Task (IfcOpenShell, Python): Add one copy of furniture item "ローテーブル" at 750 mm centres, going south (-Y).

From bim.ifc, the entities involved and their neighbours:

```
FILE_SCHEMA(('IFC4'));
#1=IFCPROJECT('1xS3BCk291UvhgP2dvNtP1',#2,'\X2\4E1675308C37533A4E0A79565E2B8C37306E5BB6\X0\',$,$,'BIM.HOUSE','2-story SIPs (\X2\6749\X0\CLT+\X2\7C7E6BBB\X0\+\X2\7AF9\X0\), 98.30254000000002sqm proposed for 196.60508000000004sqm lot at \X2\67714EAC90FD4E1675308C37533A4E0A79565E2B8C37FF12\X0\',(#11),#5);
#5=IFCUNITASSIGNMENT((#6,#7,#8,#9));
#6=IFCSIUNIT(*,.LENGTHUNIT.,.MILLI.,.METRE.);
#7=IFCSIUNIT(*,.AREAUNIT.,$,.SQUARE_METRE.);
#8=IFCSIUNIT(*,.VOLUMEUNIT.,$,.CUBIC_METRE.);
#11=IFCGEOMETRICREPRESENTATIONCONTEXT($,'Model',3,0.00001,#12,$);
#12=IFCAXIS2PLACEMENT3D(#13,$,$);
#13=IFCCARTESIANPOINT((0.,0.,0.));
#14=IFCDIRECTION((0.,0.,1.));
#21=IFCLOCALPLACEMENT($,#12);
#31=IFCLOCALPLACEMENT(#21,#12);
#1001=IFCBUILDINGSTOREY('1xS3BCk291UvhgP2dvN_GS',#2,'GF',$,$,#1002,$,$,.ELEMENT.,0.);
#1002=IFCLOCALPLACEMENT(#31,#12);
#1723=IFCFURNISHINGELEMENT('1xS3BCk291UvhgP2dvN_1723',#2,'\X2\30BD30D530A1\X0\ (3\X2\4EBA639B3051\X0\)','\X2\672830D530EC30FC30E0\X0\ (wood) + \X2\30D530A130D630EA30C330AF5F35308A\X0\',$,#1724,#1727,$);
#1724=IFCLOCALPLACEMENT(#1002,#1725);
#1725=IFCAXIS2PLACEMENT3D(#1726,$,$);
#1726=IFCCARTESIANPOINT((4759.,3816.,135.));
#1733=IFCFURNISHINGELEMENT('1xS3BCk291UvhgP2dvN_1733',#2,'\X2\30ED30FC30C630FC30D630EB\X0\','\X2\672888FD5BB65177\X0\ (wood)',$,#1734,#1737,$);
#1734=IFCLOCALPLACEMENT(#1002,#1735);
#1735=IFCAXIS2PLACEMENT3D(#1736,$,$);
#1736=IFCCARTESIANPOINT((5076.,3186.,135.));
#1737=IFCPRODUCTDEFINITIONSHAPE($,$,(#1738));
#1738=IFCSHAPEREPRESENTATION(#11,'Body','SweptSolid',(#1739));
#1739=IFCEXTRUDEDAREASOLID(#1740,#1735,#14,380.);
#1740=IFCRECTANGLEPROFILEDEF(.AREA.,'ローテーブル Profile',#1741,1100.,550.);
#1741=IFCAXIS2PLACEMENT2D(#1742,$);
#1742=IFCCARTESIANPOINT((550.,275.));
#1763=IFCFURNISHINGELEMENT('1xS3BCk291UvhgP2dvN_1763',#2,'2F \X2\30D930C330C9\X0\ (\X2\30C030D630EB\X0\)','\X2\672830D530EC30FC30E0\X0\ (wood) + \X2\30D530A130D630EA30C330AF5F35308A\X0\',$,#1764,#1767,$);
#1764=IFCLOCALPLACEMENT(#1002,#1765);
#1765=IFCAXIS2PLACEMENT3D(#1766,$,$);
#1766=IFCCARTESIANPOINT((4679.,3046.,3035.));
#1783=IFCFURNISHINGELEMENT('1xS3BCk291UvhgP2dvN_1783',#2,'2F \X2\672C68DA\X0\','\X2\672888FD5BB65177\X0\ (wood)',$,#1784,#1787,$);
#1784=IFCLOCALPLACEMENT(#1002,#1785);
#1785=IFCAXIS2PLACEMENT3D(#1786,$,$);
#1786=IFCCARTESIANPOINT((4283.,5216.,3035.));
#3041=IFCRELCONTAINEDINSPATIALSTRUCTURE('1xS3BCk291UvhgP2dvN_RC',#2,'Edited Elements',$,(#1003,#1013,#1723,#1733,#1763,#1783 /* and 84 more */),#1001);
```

```python
import numpy as np
import ifcopenshell
import ifcopenshell.api.geometry
import ifcopenshell.api.root
import ifcopenshell.util.element
import ifcopenshell.util.placement

model = ifcopenshell.open("bim.ifc")


def reuse_history(source, copy):
    """copy_class also copies each property set's owner history, people and application; keep the originals."""
    for rel in copy.IsDefinedBy:
        if rel.is_a("IfcRelDefinesByProperties") and (history := rel.RelatingPropertyDefinition.OwnerHistory):
            rel.RelatingPropertyDefinition.OwnerHistory = source.OwnerHistory
            ifcopenshell.util.element.remove_deep2(model, history)


source = model.by_guid("1xS3BCk291UvhgP2dvN_1733")
base = ifcopenshell.util.placement.get_local_placement(source.ObjectPlacement)
step = np.array([0.0, -1.0, 0.0]) * 750.0

for i in range(1, 2):
    copy = ifcopenshell.api.root.copy_class(model, product=source)
    copy.Representation = ifcopenshell.util.element.copy_deep(
        model, source.Representation, exclude=["IfcGeometricRepresentationContext", "IfcRepresentationMap"]
    )
    reuse_history(source, copy)
    matrix = base.copy()
    matrix[:3, 3] += i * step
    print("added at", matrix[:3, 3].round(3) + 0.0)
    ifcopenshell.api.geometry.edit_object_placement(model, product=copy, matrix=matrix, is_si=False)

model.write("bim_rev.ifc")
```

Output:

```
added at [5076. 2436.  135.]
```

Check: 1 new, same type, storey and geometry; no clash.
